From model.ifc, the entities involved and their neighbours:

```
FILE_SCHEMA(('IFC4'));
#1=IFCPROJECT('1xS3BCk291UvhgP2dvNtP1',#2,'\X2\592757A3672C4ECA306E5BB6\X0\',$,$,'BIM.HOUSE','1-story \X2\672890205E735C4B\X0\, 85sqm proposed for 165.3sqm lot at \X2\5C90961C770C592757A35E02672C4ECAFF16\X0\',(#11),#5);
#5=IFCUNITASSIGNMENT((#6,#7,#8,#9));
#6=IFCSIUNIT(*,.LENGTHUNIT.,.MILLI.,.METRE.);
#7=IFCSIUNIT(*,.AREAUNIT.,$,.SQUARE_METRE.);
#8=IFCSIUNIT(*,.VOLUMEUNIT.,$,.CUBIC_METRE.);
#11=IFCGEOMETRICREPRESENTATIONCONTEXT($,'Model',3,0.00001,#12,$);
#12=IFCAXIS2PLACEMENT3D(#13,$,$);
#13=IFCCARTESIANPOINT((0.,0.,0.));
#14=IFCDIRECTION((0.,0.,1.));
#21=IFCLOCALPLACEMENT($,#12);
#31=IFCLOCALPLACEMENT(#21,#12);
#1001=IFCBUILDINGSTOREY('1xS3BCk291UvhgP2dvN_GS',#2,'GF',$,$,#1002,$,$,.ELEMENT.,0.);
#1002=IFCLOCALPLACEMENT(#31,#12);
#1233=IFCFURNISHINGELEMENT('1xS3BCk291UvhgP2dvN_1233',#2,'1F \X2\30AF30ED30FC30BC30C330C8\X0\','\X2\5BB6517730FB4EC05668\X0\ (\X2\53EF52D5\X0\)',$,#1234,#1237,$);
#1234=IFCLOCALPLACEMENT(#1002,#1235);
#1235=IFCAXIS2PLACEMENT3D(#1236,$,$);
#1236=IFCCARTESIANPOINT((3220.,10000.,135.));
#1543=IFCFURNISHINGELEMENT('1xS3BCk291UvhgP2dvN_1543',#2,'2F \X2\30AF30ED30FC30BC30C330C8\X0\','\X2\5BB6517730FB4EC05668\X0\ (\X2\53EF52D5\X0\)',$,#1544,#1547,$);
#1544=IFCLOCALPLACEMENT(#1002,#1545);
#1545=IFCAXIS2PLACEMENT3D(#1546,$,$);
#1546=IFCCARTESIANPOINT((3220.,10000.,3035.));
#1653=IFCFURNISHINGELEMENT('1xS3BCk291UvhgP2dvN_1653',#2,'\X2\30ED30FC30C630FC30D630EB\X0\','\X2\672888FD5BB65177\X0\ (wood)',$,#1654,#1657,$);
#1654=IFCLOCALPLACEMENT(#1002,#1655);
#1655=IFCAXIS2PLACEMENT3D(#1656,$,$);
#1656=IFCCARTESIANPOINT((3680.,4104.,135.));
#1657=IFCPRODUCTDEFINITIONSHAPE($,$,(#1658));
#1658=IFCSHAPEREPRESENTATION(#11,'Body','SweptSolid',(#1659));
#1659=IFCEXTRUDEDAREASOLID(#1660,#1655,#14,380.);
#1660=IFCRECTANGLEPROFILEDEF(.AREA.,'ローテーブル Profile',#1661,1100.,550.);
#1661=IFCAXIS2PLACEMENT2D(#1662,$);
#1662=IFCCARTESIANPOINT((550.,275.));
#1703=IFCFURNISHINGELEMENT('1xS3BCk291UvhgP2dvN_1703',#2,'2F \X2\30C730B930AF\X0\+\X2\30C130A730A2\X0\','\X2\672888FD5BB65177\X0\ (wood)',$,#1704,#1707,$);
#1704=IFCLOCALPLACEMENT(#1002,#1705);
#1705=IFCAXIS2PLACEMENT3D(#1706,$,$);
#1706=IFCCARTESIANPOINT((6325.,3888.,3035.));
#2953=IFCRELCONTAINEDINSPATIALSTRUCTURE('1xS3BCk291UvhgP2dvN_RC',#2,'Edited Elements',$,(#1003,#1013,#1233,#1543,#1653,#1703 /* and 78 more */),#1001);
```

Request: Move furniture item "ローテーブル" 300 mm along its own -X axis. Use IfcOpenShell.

```python
import ifcopenshell
import ifcopenshell.api.geometry
import ifcopenshell.util.placement
import ifcopenshell.util.unit

model = ifcopenshell.open("model.ifc")
unit_scale = ifcopenshell.util.unit.calculate_unit_scale(model)

item = model.by_id(1653)
matrix = ifcopenshell.util.placement.get_local_placement(item.ObjectPlacement)
matrix[:3, 3] -= matrix[:3, 0] * 0.3 / unit_scale
ifcopenshell.api.geometry.edit_object_placement(model, product=item, matrix=matrix, is_si=False)

print(ifcopenshell.util.placement.get_local_placement(item.ObjectPlacement).round(3) + 0.0)

model.write("model_updated.ifc")
```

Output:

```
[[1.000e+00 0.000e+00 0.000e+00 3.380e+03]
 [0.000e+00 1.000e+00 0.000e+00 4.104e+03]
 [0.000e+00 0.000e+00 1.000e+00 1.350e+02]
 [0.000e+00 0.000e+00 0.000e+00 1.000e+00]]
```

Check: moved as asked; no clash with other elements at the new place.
